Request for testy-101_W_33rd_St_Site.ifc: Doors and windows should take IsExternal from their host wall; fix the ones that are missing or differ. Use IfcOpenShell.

First a look at what the model holds.

```python
import ifcopenshell
import ifcopenshell.util.element

model = ifcopenshell.open("testy-101_W_33rd_St_Site.ifc")
print(model.schema)
seen = {}
for e in model.by_type("IfcDoor") + model.by_type("IfcWindow"):
    if not e.FillsVoids:
        continue
    host = e.FillsVoids[0].RelatingOpeningElement.VoidsElements[0].RelatingBuildingElement
    own = ifcopenshell.util.element.get_pset(e, f"Pset_{e.is_a()[3:].removesuffix('StandardCase')}Common", "IsExternal")
    wall = ifcopenshell.util.element.get_pset(host, "Pset_WallCommon", "IsExternal")
    seen[e.is_a(), own, wall] = seen.get((e.is_a(), own, wall), 0) + 1
for (cls, own, wall), count in sorted(seen.items(), key=str):
    print(count, cls, "IsExternal:", own, "| host wall:", wall)
```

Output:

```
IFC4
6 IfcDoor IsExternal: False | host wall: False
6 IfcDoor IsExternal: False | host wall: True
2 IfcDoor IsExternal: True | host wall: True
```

```python
import ifcopenshell
import ifcopenshell.api.pset
import ifcopenshell.util.element

model = ifcopenshell.open("testy-101_W_33rd_St_Site.ifc")

count = 0
for ifc_class, pset_name in (("IfcDoor", "Pset_DoorCommon"), ("IfcWindow", "Pset_WindowCommon")):
    for e in model.by_type(ifc_class):
        if not e.FillsVoids:
            continue
        host = e.FillsVoids[0].RelatingOpeningElement.VoidsElements[0].RelatingBuildingElement
        external = ifcopenshell.util.element.get_pset(host, "Pset_WallCommon", "IsExternal")
        if external is None or ifcopenshell.util.element.get_pset(e, pset_name, "IsExternal") == external:
            continue
        pset = ifcopenshell.api.pset.add_pset(model, product=e, name=pset_name)
        ifcopenshell.api.pset.edit_pset(model, pset=pset, properties={"IsExternal": external})
        count += 1

print(count, "updated")

model.write("testy-101_W_33rd_St_Site_updated.ifc")
```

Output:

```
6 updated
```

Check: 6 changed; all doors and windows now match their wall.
